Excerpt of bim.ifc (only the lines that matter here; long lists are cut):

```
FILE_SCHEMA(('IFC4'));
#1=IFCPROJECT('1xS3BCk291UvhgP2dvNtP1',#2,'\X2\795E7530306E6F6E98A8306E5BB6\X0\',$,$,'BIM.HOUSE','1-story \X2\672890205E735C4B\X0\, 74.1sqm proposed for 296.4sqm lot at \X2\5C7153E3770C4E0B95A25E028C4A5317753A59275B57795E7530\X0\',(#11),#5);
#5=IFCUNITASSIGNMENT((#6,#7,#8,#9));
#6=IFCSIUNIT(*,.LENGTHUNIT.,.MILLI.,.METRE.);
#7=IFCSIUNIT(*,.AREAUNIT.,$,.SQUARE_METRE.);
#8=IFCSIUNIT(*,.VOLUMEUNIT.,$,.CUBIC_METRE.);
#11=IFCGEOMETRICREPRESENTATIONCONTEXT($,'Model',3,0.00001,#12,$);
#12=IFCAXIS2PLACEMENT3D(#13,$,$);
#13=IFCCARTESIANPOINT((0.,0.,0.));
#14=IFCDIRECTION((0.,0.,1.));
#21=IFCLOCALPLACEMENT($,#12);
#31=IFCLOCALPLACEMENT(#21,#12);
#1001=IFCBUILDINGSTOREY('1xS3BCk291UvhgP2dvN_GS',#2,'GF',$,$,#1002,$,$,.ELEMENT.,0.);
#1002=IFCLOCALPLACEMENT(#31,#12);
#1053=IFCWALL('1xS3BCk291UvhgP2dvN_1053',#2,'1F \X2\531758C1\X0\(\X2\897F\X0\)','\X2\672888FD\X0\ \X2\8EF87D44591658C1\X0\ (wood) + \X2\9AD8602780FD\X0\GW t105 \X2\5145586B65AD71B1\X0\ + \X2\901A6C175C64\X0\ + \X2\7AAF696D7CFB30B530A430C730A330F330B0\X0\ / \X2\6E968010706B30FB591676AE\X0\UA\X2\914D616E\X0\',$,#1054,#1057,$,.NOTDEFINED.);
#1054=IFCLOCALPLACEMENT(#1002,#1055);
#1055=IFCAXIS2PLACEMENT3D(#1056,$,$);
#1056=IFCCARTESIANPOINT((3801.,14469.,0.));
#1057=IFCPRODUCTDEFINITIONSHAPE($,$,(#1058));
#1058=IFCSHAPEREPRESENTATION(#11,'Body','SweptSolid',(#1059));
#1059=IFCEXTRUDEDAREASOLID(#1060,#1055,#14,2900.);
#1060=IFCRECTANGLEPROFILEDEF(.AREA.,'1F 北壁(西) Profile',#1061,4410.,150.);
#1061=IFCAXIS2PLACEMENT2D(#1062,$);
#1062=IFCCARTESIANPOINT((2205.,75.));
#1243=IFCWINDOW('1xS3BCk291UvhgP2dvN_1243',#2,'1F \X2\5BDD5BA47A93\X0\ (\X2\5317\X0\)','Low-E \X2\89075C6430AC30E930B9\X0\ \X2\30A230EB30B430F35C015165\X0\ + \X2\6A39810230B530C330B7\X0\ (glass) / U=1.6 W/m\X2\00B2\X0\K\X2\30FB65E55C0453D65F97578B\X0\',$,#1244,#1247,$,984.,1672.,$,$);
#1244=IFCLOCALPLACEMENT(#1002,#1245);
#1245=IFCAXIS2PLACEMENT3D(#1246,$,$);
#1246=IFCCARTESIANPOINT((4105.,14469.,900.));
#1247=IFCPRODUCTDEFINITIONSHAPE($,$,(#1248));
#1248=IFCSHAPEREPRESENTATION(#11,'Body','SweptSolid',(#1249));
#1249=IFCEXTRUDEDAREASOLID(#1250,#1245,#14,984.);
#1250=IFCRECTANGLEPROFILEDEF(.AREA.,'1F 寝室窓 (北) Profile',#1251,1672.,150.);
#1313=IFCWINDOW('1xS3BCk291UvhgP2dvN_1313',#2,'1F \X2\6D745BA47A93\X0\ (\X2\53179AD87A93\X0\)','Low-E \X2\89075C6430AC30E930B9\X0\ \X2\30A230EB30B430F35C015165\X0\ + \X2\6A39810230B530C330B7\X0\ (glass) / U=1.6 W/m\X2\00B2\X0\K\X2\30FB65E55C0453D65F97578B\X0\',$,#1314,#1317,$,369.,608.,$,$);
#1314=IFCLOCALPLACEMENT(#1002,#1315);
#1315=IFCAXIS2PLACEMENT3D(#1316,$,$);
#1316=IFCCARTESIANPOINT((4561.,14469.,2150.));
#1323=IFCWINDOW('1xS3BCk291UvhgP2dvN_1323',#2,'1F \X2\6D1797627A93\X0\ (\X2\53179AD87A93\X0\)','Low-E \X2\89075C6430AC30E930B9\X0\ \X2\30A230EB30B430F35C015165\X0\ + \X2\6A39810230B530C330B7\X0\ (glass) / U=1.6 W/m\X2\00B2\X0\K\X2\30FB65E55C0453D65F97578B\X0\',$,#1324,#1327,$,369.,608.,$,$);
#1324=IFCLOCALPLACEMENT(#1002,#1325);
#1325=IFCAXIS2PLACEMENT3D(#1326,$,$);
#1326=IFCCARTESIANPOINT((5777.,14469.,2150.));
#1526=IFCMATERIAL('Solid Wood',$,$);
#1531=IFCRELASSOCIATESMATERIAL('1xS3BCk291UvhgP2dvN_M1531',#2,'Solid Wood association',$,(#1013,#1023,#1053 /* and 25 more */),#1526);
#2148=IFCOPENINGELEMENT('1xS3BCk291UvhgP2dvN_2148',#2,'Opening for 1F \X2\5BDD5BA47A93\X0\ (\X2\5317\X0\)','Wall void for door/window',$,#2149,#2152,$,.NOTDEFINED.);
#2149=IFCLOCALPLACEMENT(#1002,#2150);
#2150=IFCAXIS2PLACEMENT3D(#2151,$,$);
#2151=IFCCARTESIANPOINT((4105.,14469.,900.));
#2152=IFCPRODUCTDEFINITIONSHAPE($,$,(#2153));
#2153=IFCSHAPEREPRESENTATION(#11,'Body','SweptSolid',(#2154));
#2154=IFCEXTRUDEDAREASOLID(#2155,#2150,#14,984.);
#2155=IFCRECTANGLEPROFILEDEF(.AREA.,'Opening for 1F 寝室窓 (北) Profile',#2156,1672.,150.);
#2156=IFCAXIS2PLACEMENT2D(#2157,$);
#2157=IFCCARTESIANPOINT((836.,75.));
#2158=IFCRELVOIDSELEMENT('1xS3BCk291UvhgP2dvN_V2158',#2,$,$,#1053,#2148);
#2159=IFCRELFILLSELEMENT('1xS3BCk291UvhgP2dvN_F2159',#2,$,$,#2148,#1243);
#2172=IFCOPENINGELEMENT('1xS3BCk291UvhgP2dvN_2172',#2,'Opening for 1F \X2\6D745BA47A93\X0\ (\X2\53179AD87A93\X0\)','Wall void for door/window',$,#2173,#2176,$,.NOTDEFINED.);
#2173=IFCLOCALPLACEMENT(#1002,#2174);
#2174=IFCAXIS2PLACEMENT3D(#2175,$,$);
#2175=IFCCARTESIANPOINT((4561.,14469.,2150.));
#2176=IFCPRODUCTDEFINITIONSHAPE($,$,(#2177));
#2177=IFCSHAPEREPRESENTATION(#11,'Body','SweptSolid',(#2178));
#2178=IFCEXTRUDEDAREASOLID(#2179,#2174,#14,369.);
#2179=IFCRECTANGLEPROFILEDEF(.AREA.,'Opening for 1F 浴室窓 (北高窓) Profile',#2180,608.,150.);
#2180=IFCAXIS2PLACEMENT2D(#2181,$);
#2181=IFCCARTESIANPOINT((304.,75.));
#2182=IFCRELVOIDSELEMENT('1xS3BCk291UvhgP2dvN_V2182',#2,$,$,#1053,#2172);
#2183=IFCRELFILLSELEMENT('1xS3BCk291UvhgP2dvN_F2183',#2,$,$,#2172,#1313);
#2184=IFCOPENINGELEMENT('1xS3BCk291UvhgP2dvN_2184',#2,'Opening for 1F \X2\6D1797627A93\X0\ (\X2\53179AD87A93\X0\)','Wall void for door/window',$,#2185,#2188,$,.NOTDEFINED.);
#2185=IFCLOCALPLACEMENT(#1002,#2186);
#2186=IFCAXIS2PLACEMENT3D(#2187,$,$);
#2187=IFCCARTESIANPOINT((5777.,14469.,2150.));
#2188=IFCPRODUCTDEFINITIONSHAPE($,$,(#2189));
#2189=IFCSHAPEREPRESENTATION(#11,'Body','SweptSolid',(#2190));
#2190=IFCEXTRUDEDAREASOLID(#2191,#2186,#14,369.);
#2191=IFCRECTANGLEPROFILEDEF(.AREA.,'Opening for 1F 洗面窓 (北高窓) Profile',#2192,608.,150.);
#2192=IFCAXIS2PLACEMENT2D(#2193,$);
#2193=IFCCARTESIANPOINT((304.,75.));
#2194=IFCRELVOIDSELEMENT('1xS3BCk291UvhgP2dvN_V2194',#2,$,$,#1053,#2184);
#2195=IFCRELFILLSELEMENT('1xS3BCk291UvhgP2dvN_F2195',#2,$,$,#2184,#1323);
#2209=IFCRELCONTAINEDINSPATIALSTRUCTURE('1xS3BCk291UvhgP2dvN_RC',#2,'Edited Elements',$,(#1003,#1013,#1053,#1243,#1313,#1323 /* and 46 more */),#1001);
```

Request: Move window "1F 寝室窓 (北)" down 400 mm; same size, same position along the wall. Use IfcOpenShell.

```python
import numpy as np
import ifcopenshell
import ifcopenshell.api.geometry
import ifcopenshell.util.placement
import ifcopenshell.util.unit

model = ifcopenshell.open("bim.ifc")
unit_scale = ifcopenshell.util.unit.calculate_unit_scale(model)

window = model.by_guid("1xS3BCk291UvhgP2dvN_1243")
opening = window.FillsVoids[0].RelatingOpeningElement
dz = -0.4 / unit_scale

shift = np.array([0.0, 0.0, dz])
# The window is not placed relative to its opening, so move both.
for product in (opening, window):
    matrix = ifcopenshell.util.placement.get_local_placement(product.ObjectPlacement)
    matrix[:3, 3] += shift
    ifcopenshell.api.geometry.edit_object_placement(model, product=product, matrix=matrix, is_si=False)

print(f"moved by {dz * unit_scale:+.3f} m")

model.write("bim_updated.ifc")
```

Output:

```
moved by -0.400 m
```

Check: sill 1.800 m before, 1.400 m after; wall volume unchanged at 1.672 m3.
